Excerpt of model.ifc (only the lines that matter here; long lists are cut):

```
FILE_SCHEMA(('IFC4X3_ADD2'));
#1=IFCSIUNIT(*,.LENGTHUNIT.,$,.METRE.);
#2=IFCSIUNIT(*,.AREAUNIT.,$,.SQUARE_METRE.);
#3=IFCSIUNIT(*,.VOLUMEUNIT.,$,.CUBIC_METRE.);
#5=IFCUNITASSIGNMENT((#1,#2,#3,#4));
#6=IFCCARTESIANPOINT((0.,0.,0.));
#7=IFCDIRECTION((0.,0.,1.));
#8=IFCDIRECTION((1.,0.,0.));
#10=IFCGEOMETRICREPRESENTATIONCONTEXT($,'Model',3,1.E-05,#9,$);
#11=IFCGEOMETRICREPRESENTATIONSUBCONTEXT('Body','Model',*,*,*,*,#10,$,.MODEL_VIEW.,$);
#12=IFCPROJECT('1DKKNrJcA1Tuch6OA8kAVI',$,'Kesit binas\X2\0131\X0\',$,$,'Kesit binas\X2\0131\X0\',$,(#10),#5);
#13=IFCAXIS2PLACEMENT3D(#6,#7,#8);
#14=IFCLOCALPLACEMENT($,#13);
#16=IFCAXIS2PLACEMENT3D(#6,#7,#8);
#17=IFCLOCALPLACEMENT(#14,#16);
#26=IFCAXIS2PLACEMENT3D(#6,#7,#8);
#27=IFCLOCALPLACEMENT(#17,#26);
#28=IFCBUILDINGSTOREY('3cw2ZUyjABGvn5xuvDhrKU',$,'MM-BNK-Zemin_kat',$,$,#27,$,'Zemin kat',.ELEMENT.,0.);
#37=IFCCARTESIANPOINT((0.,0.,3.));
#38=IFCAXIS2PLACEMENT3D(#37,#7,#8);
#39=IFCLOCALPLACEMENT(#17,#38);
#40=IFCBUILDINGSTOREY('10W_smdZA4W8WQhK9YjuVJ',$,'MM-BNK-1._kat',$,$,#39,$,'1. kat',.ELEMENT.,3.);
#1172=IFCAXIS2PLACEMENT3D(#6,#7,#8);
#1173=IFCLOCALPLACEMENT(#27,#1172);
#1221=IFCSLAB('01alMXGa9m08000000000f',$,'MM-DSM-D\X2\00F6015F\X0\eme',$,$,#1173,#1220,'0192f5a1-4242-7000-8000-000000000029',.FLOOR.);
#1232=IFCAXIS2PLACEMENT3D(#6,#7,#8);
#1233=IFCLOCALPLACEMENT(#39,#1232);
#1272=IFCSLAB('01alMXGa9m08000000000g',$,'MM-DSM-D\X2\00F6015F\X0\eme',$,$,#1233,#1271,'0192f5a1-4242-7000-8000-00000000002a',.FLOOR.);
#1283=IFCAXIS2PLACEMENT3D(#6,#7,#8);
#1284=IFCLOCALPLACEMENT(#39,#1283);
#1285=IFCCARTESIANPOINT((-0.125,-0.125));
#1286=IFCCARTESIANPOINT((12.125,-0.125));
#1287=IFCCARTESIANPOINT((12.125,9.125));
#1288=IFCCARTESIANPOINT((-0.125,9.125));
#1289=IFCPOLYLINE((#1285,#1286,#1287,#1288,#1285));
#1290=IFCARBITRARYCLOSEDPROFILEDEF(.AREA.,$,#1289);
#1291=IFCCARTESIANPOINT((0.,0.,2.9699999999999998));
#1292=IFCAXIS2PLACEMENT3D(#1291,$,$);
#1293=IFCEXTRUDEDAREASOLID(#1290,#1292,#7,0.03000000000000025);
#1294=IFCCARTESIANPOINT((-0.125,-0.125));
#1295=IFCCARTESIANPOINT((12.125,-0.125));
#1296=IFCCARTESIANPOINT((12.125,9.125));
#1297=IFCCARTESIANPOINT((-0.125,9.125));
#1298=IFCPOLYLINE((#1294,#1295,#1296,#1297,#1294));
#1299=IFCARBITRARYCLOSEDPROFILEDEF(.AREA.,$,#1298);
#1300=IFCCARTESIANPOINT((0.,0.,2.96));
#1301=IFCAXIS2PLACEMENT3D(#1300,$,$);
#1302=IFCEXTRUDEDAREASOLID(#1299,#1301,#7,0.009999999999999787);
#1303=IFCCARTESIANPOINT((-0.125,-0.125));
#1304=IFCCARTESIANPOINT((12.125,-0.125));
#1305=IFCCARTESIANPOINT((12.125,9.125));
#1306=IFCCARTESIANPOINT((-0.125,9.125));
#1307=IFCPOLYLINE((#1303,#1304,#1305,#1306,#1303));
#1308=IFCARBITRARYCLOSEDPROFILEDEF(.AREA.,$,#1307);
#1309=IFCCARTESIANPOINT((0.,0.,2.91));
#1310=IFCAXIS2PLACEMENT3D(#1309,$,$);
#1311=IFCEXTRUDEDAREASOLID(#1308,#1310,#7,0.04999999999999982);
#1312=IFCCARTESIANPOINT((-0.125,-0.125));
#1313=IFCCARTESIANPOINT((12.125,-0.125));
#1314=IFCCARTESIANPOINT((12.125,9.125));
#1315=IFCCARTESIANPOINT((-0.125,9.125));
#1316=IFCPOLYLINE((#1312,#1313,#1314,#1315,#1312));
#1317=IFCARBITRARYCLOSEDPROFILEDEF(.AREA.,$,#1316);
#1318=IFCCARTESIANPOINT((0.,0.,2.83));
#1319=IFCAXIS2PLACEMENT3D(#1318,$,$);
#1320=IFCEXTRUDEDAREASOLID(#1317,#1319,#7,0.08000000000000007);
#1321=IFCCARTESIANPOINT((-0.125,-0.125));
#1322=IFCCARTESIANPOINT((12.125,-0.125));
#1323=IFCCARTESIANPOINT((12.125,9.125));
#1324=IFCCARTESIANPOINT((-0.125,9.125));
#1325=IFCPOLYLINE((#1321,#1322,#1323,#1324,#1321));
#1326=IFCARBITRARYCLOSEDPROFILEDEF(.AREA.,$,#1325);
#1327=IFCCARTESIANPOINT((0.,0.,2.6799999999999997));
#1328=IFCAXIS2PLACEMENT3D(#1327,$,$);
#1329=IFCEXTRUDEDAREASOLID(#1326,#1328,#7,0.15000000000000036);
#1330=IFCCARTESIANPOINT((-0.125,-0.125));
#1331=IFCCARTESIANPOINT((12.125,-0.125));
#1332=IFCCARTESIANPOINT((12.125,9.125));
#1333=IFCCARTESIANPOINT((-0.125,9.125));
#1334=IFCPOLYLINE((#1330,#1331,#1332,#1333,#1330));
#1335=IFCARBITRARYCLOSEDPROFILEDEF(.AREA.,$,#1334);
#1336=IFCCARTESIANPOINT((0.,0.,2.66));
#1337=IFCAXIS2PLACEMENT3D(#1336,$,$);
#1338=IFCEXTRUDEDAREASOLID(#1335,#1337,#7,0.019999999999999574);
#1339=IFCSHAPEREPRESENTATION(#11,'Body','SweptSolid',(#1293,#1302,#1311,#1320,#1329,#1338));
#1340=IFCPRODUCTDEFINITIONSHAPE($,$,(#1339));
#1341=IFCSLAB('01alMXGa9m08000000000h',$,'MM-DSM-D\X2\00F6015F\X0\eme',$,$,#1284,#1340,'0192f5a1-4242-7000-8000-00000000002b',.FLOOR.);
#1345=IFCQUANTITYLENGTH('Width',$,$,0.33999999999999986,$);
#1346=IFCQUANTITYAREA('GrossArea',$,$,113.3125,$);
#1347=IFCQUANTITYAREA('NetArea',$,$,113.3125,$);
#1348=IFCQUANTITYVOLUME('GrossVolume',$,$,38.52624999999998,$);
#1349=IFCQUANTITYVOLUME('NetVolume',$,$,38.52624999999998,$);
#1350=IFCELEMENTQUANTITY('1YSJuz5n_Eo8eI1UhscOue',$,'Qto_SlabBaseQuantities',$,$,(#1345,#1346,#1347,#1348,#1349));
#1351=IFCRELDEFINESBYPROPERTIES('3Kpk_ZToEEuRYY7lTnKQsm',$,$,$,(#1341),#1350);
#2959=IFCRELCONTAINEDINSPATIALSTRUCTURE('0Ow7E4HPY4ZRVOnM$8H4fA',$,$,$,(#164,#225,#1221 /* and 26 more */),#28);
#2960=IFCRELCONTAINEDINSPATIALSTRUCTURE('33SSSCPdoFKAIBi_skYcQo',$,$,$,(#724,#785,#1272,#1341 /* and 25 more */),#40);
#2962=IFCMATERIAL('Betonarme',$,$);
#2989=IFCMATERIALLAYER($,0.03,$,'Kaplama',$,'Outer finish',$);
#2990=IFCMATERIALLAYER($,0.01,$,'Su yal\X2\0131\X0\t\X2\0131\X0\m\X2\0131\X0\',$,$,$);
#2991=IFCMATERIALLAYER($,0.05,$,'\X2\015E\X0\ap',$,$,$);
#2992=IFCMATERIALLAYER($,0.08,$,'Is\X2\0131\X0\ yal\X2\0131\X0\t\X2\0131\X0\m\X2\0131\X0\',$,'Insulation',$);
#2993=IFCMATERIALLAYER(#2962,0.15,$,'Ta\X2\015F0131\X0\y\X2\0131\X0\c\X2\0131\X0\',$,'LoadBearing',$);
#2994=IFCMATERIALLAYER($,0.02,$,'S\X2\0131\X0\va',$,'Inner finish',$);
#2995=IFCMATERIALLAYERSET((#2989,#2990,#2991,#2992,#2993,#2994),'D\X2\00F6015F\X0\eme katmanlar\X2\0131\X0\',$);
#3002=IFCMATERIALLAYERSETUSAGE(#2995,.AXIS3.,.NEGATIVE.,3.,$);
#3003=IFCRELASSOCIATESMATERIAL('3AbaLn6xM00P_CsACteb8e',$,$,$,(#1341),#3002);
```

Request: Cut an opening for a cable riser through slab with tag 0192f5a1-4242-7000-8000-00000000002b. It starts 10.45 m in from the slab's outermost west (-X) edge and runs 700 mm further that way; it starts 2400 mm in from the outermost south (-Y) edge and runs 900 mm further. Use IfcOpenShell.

```python
import numpy as np
import ifcopenshell
import ifcopenshell.api.feature
import ifcopenshell.api.geometry
import ifcopenshell.api.pset
import ifcopenshell.api.root
import ifcopenshell.geom
import ifcopenshell.util.element
import ifcopenshell.util.placement
import ifcopenshell.util.representation
import ifcopenshell.util.shape
import ifcopenshell.util.unit

model = ifcopenshell.open("model.ifc")
unit_scale = ifcopenshell.util.unit.calculate_unit_scale(model)
area_scale = ifcopenshell.util.unit.calculate_unit_scale(model, "AREAUNIT")
volume_scale = ifcopenshell.util.unit.calculate_unit_scale(model, "VOLUMEUNIT")
settings = ifcopenshell.geom.settings()


def volume(element):
    """Net volume in cubic metres, openings subtracted."""
    shape = ifcopenshell.geom.create_shape(settings, element)
    return ifcopenshell.util.shape.get_volume(shape.geometry)


slab = model.by_id(1341)
before = volume(slab)

# Extent in the slab's own axes, in metres. The edges named are its -X and -Y sides.
slab_shape = ifcopenshell.geom.create_shape(settings, slab)
vertices = ifcopenshell.util.shape.get_vertices(slab_shape.geometry)
x_min, y_min, bottom = vertices.min(axis=0)
top = vertices[:, 2].max()

opening = ifcopenshell.api.root.create_entity(model, ifc_class="IfcOpeningElement", name="Cable riser opening", predefined_type="OPENING")
context = ifcopenshell.util.representation.get_context(model, "Model", "Body", "MODEL_VIEW")
width, depth = 0.7, 0.9
outline = [(0.0, 0.0), (width, 0.0), (width, depth), (0.0, depth), (0.0, 0.0)]
# Overshoot both faces by 50 mm so the cut is clean.
shape = ifcopenshell.api.geometry.add_slab_representation(
    model, context=context, depth=top - bottom + 0.1, polyline=outline
)
ifcopenshell.api.geometry.assign_representation(model, product=opening, representation=shape)

matrix = ifcopenshell.util.placement.get_local_placement(slab.ObjectPlacement)
matrix[:, 3] = matrix @ np.append(np.array([x_min + 10.45, y_min + 2.4, bottom - 0.05]) / unit_scale, 1.0)
ifcopenshell.api.geometry.edit_object_placement(model, product=opening, matrix=matrix, is_si=False)
ifcopenshell.api.feature.add_feature(model, feature=opening, element=slab)

after = volume(slab)

# Update the slab's stored quantities.
qto = model.by_id(ifcopenshell.util.element.get_pset(slab, "Qto_SlabBaseQuantities", should_inherit=False)["id"])
ifcopenshell.api.pset.edit_qto(model, qto=qto, properties={
    "NetArea": after / (top - bottom) / area_scale,
    "NetVolume": after / volume_scale,
})

print(f"slab volume {before:.3f} -> {after:.3f} m3")

model.write("model_edited.ifc")
```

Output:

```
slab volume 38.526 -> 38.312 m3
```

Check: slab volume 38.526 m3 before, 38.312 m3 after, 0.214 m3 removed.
